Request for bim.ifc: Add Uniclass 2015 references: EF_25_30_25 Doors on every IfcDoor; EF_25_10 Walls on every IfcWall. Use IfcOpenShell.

First a look at what the model holds.

```python
import ifcopenshell

model = ifcopenshell.open("bim.ifc")
print(model.schema)
print("classifications:", [c.Name for c in model.by_type("IfcClassification")])
for ifc_class in ("IfcDoor", "IfcRoof", "IfcStair", "IfcWall", "IfcWindow"):
    print(ifc_class, len(model.by_type(ifc_class)))
```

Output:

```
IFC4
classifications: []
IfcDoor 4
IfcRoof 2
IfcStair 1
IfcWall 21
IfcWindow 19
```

```python
import ifcopenshell
import ifcopenshell.api.classification

model = ifcopenshell.open("bim.ifc")

system = ifcopenshell.api.classification.add_classification(model, classification="Uniclass 2015")

codes = {
    "IfcDoor": ("EF_25_30_25", "Doors"),
    "IfcWall": ("EF_25_10", "Walls"),
}
for ifc_class, (code, name) in codes.items():
    products = model.by_type(ifc_class)
    ifcopenshell.api.classification.add_reference(
        model, products=products, classification=system, identification=code, name=name
    )
    print(code, len(products))

model.write("bim_edited.ifc")
```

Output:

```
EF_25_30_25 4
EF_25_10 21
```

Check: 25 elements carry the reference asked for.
